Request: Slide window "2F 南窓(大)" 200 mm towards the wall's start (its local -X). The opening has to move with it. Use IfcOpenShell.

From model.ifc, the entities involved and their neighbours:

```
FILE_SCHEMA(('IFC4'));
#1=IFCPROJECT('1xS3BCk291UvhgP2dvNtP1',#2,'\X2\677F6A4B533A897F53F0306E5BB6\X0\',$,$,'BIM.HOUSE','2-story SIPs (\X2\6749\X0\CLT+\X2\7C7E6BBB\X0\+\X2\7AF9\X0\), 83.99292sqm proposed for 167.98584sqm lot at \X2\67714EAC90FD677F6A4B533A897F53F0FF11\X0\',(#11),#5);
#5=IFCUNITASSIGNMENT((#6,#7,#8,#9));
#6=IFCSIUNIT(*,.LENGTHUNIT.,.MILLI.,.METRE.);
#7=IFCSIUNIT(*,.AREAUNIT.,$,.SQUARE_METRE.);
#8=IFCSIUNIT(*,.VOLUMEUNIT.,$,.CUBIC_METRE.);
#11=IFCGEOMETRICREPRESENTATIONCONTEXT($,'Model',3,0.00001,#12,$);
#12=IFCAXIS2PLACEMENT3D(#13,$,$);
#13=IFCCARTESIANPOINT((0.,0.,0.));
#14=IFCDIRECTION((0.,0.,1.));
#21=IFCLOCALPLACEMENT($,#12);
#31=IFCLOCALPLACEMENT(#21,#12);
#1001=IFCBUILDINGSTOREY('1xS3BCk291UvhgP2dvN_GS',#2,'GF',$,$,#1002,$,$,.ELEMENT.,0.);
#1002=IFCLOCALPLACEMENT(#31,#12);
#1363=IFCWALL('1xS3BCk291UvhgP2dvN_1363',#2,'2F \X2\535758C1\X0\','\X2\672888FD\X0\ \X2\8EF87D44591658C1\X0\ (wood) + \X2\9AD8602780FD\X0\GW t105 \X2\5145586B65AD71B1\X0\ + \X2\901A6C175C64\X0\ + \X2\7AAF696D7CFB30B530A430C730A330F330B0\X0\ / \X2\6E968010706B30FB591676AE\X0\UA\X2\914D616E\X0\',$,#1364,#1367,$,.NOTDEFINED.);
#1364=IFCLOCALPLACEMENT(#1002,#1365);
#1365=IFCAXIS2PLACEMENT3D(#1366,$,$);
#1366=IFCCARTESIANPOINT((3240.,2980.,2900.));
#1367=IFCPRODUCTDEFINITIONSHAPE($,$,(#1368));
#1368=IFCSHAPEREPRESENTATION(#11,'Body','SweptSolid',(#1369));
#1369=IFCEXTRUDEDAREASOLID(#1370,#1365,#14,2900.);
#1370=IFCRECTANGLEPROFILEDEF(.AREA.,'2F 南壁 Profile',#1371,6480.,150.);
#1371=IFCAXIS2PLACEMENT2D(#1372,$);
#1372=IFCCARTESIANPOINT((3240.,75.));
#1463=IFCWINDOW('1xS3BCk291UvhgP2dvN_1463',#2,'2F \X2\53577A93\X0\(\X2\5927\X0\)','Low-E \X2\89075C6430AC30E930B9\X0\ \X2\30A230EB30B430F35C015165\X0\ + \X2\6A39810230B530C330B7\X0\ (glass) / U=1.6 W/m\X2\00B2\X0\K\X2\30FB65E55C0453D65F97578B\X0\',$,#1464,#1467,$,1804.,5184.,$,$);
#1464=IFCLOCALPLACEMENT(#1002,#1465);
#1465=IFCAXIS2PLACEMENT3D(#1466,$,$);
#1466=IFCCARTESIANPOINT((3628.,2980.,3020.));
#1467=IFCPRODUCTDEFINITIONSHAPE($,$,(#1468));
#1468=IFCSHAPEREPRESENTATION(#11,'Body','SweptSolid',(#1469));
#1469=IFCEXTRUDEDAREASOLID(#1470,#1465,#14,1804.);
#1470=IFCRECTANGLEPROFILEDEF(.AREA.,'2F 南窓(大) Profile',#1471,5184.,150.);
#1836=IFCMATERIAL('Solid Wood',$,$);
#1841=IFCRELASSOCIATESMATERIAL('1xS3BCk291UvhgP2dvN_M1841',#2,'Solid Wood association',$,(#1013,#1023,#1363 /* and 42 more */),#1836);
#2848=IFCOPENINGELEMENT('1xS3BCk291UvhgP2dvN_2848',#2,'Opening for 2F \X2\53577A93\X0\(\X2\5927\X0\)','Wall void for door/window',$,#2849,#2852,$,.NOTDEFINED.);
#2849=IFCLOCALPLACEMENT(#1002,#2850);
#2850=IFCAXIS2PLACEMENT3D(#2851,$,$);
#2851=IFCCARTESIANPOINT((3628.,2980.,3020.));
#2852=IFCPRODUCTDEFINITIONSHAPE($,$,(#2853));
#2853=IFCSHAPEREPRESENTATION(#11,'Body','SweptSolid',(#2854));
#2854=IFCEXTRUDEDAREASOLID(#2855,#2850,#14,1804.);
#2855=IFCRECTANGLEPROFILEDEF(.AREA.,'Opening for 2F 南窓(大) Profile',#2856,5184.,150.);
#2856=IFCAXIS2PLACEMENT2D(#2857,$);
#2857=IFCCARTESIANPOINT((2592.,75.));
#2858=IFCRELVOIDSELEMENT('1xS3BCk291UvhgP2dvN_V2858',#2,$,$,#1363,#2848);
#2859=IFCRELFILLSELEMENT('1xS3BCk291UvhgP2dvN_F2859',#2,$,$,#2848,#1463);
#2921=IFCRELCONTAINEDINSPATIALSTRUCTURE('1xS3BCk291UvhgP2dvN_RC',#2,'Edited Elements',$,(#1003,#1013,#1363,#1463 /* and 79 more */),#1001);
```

```python
import ifcopenshell
import ifcopenshell.api.geometry
import ifcopenshell.util.placement

model = ifcopenshell.open("model.ifc")

window = model.by_guid("1xS3BCk291UvhgP2dvN_1463")
opening = window.FillsVoids[0].RelatingOpeningElement
wall = opening.VoidsElements[0].RelatingBuildingElement

wall_matrix = ifcopenshell.util.placement.get_local_placement(wall.ObjectPlacement)
shift = wall_matrix[:3, 0] * -200.0
before = ifcopenshell.util.placement.get_local_placement(window.ObjectPlacement)[:3, 3].copy()

# The window is not placed relative to its opening, so move both.
for product in (opening, window):
    matrix = ifcopenshell.util.placement.get_local_placement(product.ObjectPlacement)
    matrix[:3, 3] += shift
    ifcopenshell.api.geometry.edit_object_placement(model, product=product, matrix=matrix, is_si=False)

after = ifcopenshell.util.placement.get_local_placement(window.ObjectPlacement)[:3, 3]
print("window moved by", (after - before).round(3) + 0.0)

model.write("model_edited.ifc")
```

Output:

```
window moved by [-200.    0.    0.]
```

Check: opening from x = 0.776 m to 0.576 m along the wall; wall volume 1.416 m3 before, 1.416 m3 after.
